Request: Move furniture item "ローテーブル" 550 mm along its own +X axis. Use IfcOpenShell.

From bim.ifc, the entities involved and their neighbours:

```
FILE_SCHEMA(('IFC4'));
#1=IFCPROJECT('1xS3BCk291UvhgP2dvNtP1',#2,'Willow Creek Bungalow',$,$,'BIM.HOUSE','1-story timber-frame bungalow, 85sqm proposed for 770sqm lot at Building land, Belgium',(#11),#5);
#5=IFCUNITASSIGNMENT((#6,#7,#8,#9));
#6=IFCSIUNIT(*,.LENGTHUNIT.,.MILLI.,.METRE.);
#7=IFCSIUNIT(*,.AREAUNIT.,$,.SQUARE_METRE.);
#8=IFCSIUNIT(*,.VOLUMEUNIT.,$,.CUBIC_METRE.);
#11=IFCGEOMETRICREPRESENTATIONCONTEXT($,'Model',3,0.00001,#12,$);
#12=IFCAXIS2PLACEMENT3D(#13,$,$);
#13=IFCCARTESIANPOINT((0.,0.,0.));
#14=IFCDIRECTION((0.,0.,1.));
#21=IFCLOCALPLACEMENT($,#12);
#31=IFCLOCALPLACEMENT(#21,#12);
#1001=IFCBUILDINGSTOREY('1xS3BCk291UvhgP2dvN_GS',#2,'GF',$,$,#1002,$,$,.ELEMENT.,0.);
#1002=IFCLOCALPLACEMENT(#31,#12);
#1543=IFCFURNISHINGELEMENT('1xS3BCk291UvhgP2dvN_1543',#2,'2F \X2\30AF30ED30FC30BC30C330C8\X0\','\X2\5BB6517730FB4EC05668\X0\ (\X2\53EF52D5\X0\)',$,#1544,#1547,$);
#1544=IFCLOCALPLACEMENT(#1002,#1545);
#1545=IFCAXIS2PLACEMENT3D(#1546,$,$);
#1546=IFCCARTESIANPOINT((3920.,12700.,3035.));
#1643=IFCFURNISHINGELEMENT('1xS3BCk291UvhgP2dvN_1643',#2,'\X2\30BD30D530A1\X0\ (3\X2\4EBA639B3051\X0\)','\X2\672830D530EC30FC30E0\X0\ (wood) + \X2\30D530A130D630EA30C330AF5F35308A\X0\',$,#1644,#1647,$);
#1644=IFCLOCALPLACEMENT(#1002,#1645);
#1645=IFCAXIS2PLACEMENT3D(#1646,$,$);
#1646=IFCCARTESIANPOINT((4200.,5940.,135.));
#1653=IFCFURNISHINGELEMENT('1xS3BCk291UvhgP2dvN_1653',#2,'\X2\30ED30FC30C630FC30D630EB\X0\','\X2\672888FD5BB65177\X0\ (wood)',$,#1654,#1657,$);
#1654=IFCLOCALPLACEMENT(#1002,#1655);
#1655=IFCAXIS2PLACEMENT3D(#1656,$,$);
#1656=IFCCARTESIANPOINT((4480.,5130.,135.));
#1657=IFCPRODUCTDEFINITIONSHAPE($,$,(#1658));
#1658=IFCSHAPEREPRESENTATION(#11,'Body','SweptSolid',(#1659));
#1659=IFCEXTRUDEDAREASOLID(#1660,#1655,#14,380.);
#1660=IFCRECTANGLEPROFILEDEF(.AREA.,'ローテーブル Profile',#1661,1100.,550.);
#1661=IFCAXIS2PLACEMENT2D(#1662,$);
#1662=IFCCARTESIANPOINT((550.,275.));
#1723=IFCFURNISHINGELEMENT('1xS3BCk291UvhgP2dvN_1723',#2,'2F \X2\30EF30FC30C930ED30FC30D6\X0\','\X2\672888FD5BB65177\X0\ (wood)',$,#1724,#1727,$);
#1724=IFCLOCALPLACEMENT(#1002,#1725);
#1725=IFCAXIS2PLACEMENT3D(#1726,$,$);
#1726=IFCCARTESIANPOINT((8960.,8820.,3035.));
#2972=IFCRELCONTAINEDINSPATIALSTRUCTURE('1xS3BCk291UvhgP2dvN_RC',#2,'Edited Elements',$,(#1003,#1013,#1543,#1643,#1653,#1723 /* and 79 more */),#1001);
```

```python
import ifcopenshell
import ifcopenshell.api.geometry
import ifcopenshell.util.placement

model = ifcopenshell.open("bim.ifc")

item = model.by_guid("1xS3BCk291UvhgP2dvN_1653")
matrix = ifcopenshell.util.placement.get_local_placement(item.ObjectPlacement)
matrix[:3, 3] += matrix[:3, 0] * 550.0
ifcopenshell.api.geometry.edit_object_placement(model, product=item, matrix=matrix, is_si=False)

print(ifcopenshell.util.placement.get_local_placement(item.ObjectPlacement).round(3) + 0.0)

model.write("bim-out.ifc")
```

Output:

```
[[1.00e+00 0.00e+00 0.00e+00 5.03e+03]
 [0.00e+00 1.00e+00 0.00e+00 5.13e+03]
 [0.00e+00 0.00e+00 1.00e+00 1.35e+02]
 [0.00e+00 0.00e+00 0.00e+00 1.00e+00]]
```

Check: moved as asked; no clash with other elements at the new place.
